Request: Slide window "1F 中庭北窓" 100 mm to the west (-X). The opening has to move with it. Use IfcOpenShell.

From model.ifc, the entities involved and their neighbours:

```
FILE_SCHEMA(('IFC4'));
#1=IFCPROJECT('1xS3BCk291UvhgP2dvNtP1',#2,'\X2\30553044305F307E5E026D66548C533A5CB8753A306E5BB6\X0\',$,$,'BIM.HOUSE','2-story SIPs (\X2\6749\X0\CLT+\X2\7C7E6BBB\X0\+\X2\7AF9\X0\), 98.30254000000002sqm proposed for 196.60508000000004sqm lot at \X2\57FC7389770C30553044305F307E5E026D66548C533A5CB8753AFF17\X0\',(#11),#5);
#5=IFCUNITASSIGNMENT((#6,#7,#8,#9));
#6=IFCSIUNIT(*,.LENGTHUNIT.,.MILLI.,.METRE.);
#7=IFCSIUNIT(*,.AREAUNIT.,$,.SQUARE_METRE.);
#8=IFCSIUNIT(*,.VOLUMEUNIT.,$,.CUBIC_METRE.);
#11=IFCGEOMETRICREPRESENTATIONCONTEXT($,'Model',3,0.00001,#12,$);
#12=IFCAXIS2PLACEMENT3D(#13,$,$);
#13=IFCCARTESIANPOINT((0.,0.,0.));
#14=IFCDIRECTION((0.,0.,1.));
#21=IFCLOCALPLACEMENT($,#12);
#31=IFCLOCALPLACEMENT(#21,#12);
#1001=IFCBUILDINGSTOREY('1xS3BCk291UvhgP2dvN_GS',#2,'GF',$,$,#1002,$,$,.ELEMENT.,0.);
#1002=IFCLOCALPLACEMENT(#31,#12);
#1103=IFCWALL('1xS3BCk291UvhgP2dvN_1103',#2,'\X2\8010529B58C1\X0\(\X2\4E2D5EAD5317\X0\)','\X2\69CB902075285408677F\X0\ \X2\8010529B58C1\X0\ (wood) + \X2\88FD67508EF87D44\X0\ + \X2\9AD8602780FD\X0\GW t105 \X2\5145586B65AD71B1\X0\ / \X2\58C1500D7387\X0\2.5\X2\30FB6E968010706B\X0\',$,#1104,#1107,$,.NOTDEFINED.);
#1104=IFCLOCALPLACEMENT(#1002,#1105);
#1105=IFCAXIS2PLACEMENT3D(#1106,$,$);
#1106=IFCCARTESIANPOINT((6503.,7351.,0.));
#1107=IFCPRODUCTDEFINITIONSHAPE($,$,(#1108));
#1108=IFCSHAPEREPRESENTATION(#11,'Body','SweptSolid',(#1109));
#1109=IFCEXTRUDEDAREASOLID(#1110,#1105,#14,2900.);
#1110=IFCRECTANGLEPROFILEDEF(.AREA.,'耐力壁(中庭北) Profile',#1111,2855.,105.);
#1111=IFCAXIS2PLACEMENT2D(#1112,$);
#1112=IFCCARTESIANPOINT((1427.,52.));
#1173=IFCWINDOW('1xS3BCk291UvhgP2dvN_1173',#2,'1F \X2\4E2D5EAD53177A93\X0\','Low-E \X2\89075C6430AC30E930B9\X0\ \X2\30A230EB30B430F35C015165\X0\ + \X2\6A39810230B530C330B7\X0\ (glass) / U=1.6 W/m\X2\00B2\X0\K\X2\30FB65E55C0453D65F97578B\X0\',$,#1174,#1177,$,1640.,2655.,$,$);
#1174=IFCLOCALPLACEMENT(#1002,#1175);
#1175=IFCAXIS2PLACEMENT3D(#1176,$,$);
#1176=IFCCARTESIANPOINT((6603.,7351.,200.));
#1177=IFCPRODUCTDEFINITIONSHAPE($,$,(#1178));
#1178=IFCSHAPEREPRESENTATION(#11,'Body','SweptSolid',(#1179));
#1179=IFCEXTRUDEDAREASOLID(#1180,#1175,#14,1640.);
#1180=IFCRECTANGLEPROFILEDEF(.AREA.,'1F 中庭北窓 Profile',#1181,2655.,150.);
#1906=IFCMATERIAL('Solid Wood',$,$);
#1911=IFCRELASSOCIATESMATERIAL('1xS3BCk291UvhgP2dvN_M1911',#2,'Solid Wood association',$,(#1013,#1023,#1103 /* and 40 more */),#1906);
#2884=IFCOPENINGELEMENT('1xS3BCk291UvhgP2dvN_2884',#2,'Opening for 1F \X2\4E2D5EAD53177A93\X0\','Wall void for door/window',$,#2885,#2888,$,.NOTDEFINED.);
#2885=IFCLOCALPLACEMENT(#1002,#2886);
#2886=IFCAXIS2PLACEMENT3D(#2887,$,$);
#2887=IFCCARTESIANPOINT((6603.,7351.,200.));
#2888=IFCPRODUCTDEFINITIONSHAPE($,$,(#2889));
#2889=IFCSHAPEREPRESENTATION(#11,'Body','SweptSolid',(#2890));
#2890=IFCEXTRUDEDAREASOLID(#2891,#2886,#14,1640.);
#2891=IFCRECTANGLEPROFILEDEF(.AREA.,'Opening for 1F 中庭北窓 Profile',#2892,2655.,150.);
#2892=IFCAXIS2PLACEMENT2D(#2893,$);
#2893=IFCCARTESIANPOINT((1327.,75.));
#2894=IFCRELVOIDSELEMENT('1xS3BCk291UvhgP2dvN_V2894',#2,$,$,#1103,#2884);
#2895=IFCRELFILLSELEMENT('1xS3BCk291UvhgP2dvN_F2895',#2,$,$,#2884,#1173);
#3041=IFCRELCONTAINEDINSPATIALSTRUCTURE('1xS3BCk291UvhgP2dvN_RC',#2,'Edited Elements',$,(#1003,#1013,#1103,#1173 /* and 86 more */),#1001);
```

```python
import ifcopenshell
import ifcopenshell.api.geometry
import ifcopenshell.util.placement

model = ifcopenshell.open("model.ifc")

window = model.by_guid("1xS3BCk291UvhgP2dvN_1173")
opening = window.FillsVoids[0].RelatingOpeningElement
wall = opening.VoidsElements[0].RelatingBuildingElement

wall_matrix = ifcopenshell.util.placement.get_local_placement(wall.ObjectPlacement)
shift = wall_matrix[:3, 0] * -100.0
before = ifcopenshell.util.placement.get_local_placement(window.ObjectPlacement)[:3, 3].copy()

# The window is not placed relative to its opening, so move both.
for product in (opening, window):
    matrix = ifcopenshell.util.placement.get_local_placement(product.ObjectPlacement)
    matrix[:3, 3] += shift
    ifcopenshell.api.geometry.edit_object_placement(model, product=product, matrix=matrix, is_si=False)

after = ifcopenshell.util.placement.get_local_placement(window.ObjectPlacement)[:3, 3]
print("window moved by", (after - before).round(3) + 0.0)

model.write("model-out.ifc")
```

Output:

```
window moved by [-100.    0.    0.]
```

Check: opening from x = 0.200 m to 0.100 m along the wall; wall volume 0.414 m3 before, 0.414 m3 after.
